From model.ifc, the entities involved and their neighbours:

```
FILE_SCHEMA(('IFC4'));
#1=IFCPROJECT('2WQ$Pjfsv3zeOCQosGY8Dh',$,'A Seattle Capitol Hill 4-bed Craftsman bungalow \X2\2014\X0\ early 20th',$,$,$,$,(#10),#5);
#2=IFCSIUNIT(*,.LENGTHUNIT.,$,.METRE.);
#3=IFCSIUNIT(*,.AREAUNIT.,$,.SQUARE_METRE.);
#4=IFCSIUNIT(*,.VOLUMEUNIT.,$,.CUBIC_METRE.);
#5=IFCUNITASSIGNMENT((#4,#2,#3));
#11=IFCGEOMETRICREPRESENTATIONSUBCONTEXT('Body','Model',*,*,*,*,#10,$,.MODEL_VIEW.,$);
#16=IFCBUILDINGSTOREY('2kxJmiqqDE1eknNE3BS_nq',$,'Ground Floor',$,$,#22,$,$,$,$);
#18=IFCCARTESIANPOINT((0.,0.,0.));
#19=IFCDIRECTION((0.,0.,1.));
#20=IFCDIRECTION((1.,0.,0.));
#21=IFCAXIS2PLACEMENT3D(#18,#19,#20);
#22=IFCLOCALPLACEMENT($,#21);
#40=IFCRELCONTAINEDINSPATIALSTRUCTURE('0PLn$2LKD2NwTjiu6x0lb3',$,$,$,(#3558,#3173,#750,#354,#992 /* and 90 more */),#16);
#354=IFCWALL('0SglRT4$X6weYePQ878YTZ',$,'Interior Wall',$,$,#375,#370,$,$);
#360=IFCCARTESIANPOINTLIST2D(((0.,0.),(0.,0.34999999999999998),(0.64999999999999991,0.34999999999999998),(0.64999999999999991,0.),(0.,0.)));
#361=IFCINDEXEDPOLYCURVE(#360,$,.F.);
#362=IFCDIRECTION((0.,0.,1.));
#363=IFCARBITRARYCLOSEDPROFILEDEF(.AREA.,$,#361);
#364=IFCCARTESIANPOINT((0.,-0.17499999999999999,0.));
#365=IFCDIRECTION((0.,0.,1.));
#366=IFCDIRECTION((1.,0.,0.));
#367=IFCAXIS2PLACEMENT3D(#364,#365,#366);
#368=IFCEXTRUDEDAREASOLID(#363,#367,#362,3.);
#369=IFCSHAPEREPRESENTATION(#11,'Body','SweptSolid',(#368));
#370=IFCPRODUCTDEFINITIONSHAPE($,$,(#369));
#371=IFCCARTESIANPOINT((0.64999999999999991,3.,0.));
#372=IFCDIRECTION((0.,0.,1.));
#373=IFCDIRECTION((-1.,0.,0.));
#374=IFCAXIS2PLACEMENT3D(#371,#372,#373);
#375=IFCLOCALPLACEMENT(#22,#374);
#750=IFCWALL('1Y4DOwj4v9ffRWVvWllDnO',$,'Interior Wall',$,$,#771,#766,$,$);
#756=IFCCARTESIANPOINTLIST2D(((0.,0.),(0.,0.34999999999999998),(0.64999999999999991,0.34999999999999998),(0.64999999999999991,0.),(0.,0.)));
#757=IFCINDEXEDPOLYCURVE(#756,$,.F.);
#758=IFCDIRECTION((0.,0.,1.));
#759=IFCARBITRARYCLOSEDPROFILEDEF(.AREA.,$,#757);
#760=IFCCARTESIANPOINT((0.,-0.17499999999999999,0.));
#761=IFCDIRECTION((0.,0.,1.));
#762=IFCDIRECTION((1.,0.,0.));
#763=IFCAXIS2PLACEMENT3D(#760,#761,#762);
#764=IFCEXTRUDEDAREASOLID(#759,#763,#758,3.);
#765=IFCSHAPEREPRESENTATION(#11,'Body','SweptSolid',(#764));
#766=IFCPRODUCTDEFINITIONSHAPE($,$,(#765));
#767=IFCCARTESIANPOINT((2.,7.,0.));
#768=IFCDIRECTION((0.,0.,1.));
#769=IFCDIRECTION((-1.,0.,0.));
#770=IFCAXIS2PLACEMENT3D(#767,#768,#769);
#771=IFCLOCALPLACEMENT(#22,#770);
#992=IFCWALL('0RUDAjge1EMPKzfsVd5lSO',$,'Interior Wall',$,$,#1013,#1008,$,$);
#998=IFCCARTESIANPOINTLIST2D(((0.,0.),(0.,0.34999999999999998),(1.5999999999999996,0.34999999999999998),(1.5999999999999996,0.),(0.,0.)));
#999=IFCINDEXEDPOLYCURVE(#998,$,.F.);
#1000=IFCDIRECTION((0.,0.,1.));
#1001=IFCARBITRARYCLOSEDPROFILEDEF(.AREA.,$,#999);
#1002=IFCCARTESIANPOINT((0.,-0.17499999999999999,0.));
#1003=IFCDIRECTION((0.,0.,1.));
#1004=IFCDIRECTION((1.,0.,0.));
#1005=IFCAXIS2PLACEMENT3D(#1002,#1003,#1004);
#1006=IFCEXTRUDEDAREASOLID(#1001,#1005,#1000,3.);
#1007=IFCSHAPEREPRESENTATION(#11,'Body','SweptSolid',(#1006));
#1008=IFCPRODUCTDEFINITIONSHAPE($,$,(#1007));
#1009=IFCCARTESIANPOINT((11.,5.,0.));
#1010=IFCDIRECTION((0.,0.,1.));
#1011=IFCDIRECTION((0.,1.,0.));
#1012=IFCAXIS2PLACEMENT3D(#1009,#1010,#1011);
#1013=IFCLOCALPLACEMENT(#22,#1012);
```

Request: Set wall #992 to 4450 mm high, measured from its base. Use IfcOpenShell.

```python
import ifcopenshell
import ifcopenshell.geom
import ifcopenshell.util.representation
import ifcopenshell.util.shape

model = ifcopenshell.open("model.ifc")
settings = ifcopenshell.geom.settings()


def volume(element):
    """Net volume in cubic metres, openings subtracted."""
    shape = ifcopenshell.geom.create_shape(settings, element)
    return ifcopenshell.util.shape.get_volume(shape.geometry)


wall = model.by_guid("0RUDAjge1EMPKzfsVd5lSO")
before = volume(wall)

body = ifcopenshell.util.representation.get_representation(wall, "Model", "Body")
solid = body.Items[0]
old_height = solid.Depth
solid.Depth = 4.45
after = volume(wall)

print(f"height {old_height:g} -> {solid.Depth:g}, volume {before:.3f} -> {after:.3f} m3")

model.write("model-out.ifc")
```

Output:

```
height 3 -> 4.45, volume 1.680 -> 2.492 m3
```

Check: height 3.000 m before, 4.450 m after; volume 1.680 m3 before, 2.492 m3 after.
